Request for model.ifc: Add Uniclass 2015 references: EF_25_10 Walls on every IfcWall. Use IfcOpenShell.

First a look at what the model holds.

```python
import ifcopenshell

model = ifcopenshell.open("model.ifc")
print(model.schema)
print("classifications:", [c.Name for c in model.by_type("IfcClassification")])
for ifc_class in ("IfcDoor", "IfcRoof", "IfcStair", "IfcWall", "IfcWindow"):
    print(ifc_class, len(model.by_type(ifc_class)))
```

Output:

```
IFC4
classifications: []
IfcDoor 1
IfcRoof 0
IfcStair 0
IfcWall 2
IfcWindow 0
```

```python
import ifcopenshell
import ifcopenshell.api.classification

model = ifcopenshell.open("model.ifc")

system = ifcopenshell.api.classification.add_classification(model, classification="Uniclass 2015")

codes = {
    "IfcWall": ("EF_25_10", "Walls"),
}
for ifc_class, (code, name) in codes.items():
    products = model.by_type(ifc_class)
    ifcopenshell.api.classification.add_reference(
        model, products=products, classification=system, identification=code, name=name
    )
    print(code, len(products))

model.write("model-out.ifc")
```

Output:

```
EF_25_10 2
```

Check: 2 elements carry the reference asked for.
